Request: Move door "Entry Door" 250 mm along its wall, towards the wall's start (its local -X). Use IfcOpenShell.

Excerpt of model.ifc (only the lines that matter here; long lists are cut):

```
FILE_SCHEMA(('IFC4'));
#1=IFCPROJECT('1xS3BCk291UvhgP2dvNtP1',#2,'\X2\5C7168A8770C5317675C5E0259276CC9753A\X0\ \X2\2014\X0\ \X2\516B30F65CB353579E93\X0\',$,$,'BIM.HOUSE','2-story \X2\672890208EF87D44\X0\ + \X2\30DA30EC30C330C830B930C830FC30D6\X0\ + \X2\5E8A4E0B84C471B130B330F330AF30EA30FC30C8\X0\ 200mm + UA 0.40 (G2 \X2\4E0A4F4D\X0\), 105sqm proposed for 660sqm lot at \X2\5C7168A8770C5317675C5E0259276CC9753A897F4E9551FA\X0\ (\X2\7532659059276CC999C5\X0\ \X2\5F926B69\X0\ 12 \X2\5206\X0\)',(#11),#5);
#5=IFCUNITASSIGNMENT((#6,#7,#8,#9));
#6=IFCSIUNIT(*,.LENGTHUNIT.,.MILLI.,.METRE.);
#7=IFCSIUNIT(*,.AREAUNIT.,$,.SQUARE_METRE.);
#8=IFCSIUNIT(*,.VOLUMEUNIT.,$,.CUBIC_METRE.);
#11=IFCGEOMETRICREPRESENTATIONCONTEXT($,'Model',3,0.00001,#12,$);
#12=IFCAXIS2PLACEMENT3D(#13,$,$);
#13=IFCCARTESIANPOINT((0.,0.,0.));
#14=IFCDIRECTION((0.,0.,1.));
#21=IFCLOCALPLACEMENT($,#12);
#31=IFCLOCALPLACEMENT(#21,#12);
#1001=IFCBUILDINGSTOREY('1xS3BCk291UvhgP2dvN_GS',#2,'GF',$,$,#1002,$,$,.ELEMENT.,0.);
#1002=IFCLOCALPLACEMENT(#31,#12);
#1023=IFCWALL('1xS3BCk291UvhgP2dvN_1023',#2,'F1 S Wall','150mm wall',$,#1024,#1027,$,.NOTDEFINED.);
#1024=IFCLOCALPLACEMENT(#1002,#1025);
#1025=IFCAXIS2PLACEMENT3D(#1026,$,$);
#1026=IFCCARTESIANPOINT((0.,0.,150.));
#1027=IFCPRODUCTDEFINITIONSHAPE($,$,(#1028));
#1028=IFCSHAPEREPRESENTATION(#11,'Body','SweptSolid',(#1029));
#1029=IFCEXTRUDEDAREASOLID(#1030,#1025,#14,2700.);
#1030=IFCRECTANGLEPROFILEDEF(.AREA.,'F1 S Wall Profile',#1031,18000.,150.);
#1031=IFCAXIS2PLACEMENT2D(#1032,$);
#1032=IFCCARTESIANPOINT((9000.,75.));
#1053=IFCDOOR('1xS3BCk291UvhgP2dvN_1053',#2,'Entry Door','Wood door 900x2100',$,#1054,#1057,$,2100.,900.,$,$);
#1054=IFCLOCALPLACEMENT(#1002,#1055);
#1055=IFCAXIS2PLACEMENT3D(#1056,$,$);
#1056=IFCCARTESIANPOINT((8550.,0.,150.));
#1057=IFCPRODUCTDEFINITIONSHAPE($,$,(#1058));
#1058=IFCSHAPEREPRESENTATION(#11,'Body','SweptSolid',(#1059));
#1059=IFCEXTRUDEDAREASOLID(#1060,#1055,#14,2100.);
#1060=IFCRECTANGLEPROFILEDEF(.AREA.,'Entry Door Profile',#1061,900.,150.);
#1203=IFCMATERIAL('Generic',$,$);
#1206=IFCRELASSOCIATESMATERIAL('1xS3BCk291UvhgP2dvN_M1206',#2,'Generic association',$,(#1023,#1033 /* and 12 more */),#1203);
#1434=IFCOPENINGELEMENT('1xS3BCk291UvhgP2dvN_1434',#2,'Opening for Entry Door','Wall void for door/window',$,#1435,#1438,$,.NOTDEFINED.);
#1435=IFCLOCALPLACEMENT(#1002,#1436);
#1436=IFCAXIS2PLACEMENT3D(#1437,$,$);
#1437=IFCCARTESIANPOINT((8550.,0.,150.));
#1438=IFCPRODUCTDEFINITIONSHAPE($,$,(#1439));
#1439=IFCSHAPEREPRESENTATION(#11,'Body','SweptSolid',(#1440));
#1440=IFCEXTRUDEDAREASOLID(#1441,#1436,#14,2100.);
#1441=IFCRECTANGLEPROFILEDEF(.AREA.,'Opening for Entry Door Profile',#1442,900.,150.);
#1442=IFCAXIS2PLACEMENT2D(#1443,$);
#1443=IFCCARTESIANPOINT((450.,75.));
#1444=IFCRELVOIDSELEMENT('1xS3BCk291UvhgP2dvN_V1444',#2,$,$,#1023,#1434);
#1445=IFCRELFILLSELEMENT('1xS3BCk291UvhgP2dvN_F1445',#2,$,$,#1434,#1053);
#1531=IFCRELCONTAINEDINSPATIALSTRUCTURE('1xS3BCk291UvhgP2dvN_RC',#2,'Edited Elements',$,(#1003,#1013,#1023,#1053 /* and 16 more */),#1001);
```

```python
import ifcopenshell
import ifcopenshell.api.geometry
import ifcopenshell.util.placement
import ifcopenshell.util.unit

model = ifcopenshell.open("model.ifc")
unit_scale = ifcopenshell.util.unit.calculate_unit_scale(model)

door = model.by_guid("1xS3BCk291UvhgP2dvN_1053")
opening = door.FillsVoids[0].RelatingOpeningElement
wall = opening.VoidsElements[0].RelatingBuildingElement

wall_matrix = ifcopenshell.util.placement.get_local_placement(wall.ObjectPlacement)
shift = wall_matrix[:3, 0] * -0.25 / unit_scale
before = ifcopenshell.util.placement.get_local_placement(door.ObjectPlacement)[:3, 3].copy()

# The door is not placed relative to its opening, so move both.
for product in (opening, door):
    matrix = ifcopenshell.util.placement.get_local_placement(product.ObjectPlacement)
    matrix[:3, 3] += shift
    ifcopenshell.api.geometry.edit_object_placement(model, product=product, matrix=matrix, is_si=False)

after = ifcopenshell.util.placement.get_local_placement(door.ObjectPlacement)[:3, 3]
print("door moved by", (after - before).round(3) + 0.0)

model.write("model_v2.ifc")
```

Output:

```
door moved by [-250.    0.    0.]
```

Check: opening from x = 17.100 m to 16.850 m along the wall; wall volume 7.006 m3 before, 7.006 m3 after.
